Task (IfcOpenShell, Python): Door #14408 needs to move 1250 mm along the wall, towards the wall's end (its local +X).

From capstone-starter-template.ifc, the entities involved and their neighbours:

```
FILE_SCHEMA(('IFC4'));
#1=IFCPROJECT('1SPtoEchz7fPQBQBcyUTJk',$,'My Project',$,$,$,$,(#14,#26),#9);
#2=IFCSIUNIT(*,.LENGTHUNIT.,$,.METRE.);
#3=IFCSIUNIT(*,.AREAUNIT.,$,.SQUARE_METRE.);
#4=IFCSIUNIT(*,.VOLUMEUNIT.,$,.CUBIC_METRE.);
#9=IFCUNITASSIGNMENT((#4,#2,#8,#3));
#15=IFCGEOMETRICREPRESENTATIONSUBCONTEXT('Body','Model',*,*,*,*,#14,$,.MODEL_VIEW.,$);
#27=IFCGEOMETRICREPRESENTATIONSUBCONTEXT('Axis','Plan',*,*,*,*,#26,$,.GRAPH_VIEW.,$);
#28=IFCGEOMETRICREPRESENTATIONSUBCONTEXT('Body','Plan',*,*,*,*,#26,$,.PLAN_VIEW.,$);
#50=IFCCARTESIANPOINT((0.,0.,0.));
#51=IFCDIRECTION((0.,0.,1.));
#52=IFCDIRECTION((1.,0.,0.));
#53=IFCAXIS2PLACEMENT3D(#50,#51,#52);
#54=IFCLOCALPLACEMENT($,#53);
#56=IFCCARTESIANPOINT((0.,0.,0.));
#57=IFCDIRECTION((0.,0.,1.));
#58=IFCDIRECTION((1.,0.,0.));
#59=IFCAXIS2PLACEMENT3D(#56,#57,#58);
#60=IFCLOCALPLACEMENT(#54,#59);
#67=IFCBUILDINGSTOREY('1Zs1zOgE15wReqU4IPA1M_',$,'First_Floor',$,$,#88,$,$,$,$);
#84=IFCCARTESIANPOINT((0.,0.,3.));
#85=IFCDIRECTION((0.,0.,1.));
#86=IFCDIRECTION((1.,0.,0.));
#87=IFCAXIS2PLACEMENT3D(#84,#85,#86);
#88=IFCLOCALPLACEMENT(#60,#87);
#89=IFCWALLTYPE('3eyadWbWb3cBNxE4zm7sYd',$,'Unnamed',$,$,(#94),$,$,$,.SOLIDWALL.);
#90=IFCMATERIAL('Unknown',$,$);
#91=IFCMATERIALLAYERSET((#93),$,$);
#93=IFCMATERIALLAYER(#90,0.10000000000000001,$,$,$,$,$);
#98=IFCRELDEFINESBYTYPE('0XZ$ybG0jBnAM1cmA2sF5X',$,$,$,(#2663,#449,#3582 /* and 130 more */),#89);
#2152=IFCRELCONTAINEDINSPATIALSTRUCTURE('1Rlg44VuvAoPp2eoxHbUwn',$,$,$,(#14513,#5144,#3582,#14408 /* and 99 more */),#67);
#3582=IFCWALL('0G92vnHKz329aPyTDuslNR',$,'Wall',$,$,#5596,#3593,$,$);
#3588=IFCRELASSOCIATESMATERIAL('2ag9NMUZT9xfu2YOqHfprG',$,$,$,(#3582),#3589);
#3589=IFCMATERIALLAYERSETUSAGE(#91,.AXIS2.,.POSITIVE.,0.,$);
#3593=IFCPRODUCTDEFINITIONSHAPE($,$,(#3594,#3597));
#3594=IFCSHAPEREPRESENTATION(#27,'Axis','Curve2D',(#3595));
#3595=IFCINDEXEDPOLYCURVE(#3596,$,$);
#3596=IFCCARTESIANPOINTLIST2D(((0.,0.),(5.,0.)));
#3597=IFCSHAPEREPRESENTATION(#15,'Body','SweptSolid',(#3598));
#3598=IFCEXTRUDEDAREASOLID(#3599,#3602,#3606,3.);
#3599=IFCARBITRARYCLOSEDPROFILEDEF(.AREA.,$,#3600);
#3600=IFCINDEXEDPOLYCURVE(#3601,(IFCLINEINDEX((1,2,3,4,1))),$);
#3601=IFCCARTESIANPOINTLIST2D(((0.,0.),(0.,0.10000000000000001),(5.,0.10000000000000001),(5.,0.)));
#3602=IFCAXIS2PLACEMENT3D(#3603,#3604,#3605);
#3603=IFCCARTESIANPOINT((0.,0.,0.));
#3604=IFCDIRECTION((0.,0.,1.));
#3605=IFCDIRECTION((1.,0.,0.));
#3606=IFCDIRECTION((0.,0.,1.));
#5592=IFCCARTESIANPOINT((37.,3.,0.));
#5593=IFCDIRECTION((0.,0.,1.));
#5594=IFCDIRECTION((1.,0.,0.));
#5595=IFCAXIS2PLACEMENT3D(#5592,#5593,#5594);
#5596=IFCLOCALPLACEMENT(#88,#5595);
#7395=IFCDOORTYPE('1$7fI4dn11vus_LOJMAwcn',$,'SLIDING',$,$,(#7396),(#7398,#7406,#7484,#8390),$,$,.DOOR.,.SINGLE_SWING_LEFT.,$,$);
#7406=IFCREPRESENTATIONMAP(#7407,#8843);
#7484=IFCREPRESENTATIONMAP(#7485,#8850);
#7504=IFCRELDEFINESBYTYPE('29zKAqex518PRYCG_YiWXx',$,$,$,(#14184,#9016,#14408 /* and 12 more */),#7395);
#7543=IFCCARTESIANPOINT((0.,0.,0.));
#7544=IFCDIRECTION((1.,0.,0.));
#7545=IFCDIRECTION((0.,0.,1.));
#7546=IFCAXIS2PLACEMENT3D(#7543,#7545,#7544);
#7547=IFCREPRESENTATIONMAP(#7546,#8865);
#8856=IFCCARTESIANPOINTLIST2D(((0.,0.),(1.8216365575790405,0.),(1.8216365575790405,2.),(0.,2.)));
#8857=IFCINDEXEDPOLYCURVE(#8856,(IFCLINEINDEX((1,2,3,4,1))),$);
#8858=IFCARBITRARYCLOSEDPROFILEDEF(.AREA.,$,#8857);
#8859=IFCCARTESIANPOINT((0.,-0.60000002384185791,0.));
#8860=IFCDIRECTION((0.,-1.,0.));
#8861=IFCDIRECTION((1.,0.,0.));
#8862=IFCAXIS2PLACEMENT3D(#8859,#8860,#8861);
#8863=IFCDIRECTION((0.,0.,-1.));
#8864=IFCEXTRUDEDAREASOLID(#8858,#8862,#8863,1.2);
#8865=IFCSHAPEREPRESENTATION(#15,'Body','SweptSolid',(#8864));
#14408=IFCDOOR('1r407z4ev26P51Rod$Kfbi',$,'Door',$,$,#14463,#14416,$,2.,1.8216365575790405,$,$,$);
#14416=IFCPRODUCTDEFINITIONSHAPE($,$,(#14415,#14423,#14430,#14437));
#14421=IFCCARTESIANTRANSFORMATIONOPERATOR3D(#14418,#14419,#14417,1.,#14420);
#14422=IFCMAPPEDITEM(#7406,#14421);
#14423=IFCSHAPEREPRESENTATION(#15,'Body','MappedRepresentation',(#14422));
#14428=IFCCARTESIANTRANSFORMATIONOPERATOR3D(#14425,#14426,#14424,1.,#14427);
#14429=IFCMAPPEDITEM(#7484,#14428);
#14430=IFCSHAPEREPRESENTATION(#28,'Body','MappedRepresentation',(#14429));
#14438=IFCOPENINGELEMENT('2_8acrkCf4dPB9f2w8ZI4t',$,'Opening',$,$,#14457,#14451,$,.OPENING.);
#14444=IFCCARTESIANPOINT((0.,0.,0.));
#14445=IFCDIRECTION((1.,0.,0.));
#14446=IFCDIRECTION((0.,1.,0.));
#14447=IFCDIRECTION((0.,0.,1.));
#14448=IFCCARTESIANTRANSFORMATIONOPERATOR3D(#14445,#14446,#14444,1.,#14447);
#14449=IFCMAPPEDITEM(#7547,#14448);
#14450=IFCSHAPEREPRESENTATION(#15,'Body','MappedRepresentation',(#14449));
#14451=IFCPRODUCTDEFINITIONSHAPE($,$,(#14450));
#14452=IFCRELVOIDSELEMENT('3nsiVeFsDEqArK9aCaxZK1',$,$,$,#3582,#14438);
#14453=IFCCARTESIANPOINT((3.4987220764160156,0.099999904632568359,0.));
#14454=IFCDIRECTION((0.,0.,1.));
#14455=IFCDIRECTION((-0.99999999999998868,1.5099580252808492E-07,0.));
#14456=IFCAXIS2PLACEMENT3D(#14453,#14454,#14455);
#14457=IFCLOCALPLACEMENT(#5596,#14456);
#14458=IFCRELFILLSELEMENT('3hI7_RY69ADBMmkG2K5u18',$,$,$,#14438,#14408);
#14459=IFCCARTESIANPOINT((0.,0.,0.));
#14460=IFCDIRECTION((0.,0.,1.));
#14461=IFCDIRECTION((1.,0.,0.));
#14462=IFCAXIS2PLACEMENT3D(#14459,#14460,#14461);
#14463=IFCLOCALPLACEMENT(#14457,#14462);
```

```python
import ifcopenshell
import ifcopenshell.api.geometry
import ifcopenshell.util.placement

model = ifcopenshell.open("capstone-starter-template.ifc")

door = model.by_guid("1r407z4ev26P51Rod$Kfbi")
opening = door.FillsVoids[0].RelatingOpeningElement
wall = opening.VoidsElements[0].RelatingBuildingElement

wall_matrix = ifcopenshell.util.placement.get_local_placement(wall.ObjectPlacement)
shift = wall_matrix[:3, 0] * 1.25
before = ifcopenshell.util.placement.get_local_placement(door.ObjectPlacement)[:3, 3].copy()

# The door is placed relative to its opening, so it follows when the opening moves.
matrix = ifcopenshell.util.placement.get_local_placement(opening.ObjectPlacement)
matrix[:3, 3] += shift
ifcopenshell.api.geometry.edit_object_placement(
    model, product=opening, matrix=matrix, is_si=False, should_transform_children=True
)

after = ifcopenshell.util.placement.get_local_placement(door.ObjectPlacement)[:3, 3]
print("door moved by", (after - before).round(3) + 0.0)

model.write("capstone-starter-template_updated.ifc")
```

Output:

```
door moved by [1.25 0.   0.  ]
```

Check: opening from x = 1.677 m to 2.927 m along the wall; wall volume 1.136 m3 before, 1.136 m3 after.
